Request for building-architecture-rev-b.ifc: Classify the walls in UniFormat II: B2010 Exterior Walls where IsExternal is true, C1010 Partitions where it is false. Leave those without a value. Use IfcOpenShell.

First a look at what the model holds.

```python
import ifcopenshell
import ifcopenshell.util.element

model = ifcopenshell.open("building-architecture-rev-b.ifc")
print(model.schema)
print("classifications:", [c.Name for c in model.by_type("IfcClassification")])
values = [ifcopenshell.util.element.get_pset(e, "Pset_WallCommon", "IsExternal") for e in model.by_type("IfcWall")]
for value in (True, False, None):
    print("IsExternal", value, values.count(value))
```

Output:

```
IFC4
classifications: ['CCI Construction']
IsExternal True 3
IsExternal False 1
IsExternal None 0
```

```python
import ifcopenshell
import ifcopenshell.api.classification
import ifcopenshell.util.element

model = ifcopenshell.open("building-architecture-rev-b.ifc")

system = ifcopenshell.api.classification.add_classification(model, classification="UniFormat II")

walls = model.by_type("IfcWall")
external = {e: ifcopenshell.util.element.get_pset(e, "Pset_WallCommon", "IsExternal") for e in walls}
for flag, code, name in ((True, "B2010", "Exterior Walls"), (False, "C1010", "Partitions")):
    products = [e for e in walls if external[e] is flag]
    ifcopenshell.api.classification.add_reference(
        model, products=products, classification=system, identification=code, name=name
    )
    print(code, len(products))

model.write("building-architecture-rev-b_v2.ifc")
```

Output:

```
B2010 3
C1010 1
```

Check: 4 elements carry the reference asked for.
